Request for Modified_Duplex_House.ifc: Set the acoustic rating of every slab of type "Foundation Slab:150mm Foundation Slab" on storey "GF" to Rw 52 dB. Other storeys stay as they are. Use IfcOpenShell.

First a look at what the model holds.

```python
import ifcopenshell
import ifcopenshell.util.element

model = ifcopenshell.open("Modified_Duplex_House.ifc")
print(model.schema)
storey = next(s for s in model.by_type("IfcBuildingStorey") if s.Name == "GF")
slabs = [e for e in ifcopenshell.util.element.get_decomposition(storey) if e.is_a("IfcSlab")]
seen = {}
for e in slabs:
    element_type = ifcopenshell.util.element.get_type(e)
    key = (element_type.Name if element_type != e and element_type else None, ifcopenshell.util.element.get_pset(e, "Pset_SlabCommon", "AcousticRating"))
    seen[key] = seen.get(key, 0) + 1
for (name, value), count in sorted(seen.items(), key=str):
    print(count, "x", name, "|", value)
```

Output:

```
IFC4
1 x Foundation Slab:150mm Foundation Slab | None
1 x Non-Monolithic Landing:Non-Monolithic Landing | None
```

```python
import ifcopenshell
import ifcopenshell.api.pset
import ifcopenshell.util.element

model = ifcopenshell.open("Modified_Duplex_House.ifc")

storey = next(s for s in model.by_type("IfcBuildingStorey") if s.Name == "GF")
slabs = [e for e in ifcopenshell.util.element.get_decomposition(storey) if e.is_a("IfcSlab")]

count = 0
for e in slabs:
    element_type = ifcopenshell.util.element.get_type(e)
    if element_type in (None, e) or element_type.Name != "Foundation Slab:150mm Foundation Slab":
        continue
    # add_pset returns the element's existing set when there is one.
    pset = ifcopenshell.api.pset.add_pset(model, product=e, name="Pset_SlabCommon")
    ifcopenshell.api.pset.edit_pset(model, pset=pset, properties={"AcousticRating": "Rw 52 dB"})
    count += 1

print(count, "slabs updated")

model.write("Modified_Duplex_House_updated.ifc")
```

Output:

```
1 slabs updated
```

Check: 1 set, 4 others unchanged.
